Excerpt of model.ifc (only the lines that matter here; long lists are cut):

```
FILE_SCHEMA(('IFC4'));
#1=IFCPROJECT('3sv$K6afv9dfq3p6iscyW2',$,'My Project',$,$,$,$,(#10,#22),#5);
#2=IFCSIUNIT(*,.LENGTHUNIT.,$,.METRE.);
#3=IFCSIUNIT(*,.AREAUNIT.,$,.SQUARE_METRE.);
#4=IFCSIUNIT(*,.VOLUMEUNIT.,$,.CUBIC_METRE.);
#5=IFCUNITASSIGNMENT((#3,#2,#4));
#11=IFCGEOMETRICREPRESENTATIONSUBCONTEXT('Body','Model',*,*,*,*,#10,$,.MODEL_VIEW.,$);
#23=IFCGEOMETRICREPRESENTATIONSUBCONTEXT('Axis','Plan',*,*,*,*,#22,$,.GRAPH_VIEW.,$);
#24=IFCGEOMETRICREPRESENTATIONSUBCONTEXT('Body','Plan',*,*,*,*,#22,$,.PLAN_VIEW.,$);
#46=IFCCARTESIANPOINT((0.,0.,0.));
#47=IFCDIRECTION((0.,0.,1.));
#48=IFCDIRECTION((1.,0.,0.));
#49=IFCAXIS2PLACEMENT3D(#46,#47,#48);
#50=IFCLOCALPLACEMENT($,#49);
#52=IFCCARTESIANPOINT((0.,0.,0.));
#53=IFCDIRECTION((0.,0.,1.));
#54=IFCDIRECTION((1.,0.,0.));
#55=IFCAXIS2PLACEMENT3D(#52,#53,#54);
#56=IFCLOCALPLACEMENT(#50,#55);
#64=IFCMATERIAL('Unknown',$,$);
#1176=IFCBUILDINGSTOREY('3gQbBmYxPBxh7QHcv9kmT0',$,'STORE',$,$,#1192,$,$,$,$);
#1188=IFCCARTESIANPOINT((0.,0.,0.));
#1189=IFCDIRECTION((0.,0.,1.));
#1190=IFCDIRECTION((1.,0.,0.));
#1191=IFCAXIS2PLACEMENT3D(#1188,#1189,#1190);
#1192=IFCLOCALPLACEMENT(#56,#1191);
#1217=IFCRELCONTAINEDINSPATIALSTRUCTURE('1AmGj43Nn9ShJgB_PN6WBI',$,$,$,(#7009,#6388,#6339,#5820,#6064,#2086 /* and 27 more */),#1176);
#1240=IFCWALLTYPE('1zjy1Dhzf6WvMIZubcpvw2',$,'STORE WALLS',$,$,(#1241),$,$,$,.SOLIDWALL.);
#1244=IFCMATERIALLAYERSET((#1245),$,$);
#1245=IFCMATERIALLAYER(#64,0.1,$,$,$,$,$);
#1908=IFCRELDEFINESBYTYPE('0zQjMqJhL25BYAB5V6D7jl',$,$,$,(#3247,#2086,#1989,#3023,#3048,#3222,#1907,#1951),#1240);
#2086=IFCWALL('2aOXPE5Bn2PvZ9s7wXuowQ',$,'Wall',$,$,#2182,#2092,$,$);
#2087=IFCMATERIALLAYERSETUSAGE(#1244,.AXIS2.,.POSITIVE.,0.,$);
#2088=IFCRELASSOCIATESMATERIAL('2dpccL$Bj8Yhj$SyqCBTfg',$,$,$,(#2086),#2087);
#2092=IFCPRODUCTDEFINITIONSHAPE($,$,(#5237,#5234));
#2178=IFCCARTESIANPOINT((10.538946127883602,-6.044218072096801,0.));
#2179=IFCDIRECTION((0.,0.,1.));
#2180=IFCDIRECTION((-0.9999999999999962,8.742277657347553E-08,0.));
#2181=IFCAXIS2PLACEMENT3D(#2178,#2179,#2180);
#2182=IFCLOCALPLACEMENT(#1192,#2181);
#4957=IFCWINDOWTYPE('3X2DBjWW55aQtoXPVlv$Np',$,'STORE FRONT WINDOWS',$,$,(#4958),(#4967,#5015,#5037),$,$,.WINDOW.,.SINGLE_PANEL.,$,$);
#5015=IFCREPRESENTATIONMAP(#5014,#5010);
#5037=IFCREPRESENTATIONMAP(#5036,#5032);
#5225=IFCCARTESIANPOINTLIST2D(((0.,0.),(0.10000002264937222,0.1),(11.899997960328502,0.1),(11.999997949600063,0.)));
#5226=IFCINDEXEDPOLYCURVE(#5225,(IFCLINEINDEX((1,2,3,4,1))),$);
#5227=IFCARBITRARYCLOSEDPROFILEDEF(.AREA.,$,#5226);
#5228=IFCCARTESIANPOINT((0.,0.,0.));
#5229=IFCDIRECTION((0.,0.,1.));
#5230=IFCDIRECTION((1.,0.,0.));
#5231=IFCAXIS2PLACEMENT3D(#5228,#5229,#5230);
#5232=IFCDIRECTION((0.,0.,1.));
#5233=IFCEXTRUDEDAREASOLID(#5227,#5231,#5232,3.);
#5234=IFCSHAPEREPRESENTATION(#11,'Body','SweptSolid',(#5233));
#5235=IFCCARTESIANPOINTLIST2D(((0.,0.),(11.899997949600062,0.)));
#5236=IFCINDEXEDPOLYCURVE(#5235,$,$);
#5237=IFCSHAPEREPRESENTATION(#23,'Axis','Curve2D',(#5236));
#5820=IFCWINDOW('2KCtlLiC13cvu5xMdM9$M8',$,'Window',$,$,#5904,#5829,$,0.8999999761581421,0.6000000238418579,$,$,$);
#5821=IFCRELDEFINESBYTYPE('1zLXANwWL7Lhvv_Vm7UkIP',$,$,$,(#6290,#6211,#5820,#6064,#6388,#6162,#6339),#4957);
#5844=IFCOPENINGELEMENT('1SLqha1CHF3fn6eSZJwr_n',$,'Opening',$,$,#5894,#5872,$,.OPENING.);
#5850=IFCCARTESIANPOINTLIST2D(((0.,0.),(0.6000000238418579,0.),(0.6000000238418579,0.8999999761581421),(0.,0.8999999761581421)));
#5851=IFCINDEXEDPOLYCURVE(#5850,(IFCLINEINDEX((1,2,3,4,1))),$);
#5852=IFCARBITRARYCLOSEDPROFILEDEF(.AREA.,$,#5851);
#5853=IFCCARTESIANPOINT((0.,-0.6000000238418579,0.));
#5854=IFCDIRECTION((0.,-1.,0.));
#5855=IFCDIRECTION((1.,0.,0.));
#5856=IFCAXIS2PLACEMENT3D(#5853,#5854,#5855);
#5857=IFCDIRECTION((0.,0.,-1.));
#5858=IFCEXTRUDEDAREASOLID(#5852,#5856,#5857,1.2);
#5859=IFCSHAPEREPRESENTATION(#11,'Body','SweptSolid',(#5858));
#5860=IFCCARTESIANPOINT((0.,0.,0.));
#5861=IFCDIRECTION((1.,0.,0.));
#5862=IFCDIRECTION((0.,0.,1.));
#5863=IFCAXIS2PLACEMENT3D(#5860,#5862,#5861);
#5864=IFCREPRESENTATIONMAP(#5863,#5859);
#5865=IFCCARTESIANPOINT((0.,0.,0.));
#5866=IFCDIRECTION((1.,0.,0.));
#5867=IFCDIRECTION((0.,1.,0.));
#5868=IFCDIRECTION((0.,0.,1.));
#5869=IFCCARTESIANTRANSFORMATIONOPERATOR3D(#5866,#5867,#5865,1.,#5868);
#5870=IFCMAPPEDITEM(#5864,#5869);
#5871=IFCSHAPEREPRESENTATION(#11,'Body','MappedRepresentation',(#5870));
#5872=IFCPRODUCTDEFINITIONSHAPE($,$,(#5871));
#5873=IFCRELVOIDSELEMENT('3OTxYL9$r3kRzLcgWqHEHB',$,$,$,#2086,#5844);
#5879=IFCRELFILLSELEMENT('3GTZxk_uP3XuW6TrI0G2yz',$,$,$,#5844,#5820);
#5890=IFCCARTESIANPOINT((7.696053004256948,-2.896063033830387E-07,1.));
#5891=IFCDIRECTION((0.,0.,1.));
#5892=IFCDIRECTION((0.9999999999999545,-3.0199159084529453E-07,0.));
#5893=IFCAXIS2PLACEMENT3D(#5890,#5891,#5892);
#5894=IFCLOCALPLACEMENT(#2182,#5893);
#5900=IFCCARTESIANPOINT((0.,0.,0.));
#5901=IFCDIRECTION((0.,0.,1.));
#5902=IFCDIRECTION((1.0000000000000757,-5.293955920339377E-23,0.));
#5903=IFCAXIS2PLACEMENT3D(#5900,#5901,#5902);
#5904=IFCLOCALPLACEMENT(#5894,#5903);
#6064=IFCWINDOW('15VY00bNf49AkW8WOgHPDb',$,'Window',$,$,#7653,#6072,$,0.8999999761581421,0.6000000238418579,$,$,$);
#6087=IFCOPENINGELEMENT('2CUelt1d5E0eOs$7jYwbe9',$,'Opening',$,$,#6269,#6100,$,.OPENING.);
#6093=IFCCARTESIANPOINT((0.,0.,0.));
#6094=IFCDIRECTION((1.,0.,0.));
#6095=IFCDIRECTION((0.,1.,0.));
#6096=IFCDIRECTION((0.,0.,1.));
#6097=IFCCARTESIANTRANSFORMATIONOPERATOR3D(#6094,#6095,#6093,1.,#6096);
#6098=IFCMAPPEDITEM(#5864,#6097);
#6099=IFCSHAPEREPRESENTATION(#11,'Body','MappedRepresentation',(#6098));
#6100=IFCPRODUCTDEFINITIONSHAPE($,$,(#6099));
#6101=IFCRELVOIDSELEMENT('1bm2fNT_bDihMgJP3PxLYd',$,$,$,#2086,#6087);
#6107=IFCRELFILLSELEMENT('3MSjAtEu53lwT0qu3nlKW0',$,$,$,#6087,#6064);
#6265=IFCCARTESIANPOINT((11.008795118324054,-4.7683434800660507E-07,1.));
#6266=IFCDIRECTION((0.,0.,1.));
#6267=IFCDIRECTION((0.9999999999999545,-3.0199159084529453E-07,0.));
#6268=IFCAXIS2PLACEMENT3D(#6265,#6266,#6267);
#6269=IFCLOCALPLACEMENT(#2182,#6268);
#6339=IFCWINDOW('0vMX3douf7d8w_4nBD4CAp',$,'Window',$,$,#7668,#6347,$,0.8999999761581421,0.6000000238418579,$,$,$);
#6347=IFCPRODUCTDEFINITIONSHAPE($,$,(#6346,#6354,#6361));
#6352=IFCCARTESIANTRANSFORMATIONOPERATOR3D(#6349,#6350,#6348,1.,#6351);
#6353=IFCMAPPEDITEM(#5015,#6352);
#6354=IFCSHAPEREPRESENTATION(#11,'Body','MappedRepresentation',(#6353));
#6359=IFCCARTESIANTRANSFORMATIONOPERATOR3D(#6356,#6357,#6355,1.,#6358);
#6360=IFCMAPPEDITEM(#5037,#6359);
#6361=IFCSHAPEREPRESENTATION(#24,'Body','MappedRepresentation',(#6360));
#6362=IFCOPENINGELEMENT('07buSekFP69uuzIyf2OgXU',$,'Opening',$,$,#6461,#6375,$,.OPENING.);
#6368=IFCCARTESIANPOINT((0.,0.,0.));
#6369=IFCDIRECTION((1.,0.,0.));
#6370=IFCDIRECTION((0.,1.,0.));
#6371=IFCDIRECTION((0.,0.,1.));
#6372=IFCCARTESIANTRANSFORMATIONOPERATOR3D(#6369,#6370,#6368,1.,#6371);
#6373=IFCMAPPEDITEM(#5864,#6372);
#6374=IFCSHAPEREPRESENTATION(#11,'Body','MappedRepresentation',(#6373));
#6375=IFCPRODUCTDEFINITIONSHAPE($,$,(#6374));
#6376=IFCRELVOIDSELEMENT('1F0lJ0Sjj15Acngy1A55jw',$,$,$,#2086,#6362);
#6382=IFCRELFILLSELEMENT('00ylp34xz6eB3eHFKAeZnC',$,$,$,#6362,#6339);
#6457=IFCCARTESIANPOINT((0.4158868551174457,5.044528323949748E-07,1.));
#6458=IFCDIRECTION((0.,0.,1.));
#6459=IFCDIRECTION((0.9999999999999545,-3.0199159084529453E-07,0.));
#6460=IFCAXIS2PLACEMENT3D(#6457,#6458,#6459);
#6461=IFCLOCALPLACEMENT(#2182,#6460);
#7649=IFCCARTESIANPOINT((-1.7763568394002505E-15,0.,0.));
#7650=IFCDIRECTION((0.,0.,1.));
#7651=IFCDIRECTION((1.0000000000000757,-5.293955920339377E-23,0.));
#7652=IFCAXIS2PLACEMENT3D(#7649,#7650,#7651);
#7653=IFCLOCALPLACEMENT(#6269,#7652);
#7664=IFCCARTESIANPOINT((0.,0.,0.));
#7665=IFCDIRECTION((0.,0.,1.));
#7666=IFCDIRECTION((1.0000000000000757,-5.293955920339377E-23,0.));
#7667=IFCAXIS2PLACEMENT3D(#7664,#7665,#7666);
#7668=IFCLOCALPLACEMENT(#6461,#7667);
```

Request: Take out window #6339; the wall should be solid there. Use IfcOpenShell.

```python
import ifcopenshell
import ifcopenshell.api.feature
import ifcopenshell.api.root
import ifcopenshell.geom
import ifcopenshell.util.shape

model = ifcopenshell.open("model.ifc")
settings = ifcopenshell.geom.settings()


def volume(element):
    """Net volume in cubic metres, openings subtracted."""
    shape = ifcopenshell.geom.create_shape(settings, element)
    return ifcopenshell.util.shape.get_volume(shape.geometry)


window = model.by_guid("0vMX3douf7d8w_4nBD4CAp")
opening = window.FillsVoids[0].RelatingOpeningElement
wall = opening.VoidsElements[0].RelatingBuildingElement
before = volume(wall)

ifcopenshell.api.root.remove_product(model, product=window)
ifcopenshell.api.feature.remove_feature(model, feature=opening)

after = volume(wall)

print(f"wall volume {before:.3f} -> {after:.3f} m3")

model.write("model_v2.ifc")
```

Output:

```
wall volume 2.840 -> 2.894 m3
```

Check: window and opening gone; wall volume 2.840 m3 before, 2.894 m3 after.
